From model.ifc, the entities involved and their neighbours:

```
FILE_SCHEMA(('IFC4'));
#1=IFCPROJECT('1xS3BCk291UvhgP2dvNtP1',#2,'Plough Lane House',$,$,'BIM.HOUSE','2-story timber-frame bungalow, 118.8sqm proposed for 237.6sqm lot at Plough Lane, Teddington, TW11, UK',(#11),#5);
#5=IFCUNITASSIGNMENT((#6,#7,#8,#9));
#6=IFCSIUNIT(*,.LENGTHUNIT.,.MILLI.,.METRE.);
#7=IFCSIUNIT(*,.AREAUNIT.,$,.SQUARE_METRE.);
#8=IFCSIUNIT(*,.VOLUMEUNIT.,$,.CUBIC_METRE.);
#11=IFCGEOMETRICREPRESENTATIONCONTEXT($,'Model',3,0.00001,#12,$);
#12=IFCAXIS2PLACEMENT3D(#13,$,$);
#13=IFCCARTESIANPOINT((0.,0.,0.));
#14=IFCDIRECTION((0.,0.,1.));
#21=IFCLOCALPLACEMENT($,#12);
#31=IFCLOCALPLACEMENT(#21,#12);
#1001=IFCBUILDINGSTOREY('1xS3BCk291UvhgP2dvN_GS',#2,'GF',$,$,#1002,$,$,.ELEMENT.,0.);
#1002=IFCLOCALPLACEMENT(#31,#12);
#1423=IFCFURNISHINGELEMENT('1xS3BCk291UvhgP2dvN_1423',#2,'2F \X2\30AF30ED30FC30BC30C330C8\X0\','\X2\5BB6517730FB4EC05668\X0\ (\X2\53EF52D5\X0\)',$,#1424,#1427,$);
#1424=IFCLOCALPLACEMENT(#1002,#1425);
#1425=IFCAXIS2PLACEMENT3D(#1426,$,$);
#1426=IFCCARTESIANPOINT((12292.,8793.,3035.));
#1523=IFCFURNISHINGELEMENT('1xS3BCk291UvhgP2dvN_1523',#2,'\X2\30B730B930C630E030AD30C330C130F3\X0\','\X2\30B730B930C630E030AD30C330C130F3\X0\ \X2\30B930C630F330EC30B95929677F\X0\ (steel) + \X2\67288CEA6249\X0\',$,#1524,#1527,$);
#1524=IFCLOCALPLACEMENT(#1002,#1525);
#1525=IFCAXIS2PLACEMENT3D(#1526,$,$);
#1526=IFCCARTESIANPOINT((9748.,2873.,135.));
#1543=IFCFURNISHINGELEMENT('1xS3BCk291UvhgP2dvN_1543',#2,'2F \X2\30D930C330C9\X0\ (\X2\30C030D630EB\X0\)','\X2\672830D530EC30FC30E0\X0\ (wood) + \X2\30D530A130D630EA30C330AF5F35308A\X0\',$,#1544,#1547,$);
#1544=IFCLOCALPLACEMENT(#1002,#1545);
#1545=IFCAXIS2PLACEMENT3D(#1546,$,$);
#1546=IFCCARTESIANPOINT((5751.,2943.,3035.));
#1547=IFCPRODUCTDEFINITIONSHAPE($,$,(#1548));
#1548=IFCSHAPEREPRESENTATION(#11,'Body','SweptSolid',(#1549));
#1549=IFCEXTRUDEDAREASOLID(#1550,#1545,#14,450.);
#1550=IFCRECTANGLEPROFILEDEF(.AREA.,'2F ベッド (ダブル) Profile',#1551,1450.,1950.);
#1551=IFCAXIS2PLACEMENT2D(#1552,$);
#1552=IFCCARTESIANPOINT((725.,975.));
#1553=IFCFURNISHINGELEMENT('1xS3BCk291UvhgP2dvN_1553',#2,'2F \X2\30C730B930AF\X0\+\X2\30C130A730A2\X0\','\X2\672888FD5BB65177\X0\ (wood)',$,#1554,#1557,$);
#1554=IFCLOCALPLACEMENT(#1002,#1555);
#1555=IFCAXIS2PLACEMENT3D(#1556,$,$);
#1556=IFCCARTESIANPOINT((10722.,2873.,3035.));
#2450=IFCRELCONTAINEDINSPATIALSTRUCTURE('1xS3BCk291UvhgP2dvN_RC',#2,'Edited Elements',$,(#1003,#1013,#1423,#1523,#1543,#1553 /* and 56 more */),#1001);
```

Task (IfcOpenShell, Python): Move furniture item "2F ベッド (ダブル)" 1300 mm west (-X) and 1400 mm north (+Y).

```python
import ifcopenshell
import ifcopenshell.api.geometry
import ifcopenshell.util.placement

model = ifcopenshell.open("model.ifc")

item = model.by_id(1543)
matrix = ifcopenshell.util.placement.get_local_placement(item.ObjectPlacement)
matrix[0, 3] -= 1300.0
matrix[1, 3] += 1400.0
ifcopenshell.api.geometry.edit_object_placement(model, product=item, matrix=matrix, is_si=False)

print(ifcopenshell.util.placement.get_local_placement(item.ObjectPlacement).round(3) + 0.0)

model.write("model_rev.ifc")
```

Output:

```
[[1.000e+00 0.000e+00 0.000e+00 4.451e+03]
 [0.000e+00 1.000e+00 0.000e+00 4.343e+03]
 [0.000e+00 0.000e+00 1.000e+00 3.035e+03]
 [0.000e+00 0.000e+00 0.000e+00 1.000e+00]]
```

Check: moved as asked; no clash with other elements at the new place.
